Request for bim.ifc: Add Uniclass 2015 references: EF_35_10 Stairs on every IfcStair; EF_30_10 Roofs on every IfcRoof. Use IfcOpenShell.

First a look at what the model holds.

```python
import ifcopenshell

model = ifcopenshell.open("bim.ifc")
print(model.schema)
print("classifications:", [c.Name for c in model.by_type("IfcClassification")])
for ifc_class in ("IfcDoor", "IfcRoof", "IfcStair", "IfcWall", "IfcWindow"):
    print(ifc_class, len(model.by_type(ifc_class)))
```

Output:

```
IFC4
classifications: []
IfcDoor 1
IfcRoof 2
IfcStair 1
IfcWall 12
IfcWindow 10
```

```python
import ifcopenshell
import ifcopenshell.api.classification

model = ifcopenshell.open("bim.ifc")

system = ifcopenshell.api.classification.add_classification(model, classification="Uniclass 2015")

codes = {
    "IfcStair": ("EF_35_10", "Stairs"),
    "IfcRoof": ("EF_30_10", "Roofs"),
}
for ifc_class, (code, name) in codes.items():
    products = model.by_type(ifc_class)
    ifcopenshell.api.classification.add_reference(
        model, products=products, classification=system, identification=code, name=name
    )
    print(code, len(products))

model.write("bim_rev.ifc")
```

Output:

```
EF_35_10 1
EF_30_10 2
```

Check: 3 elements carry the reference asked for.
